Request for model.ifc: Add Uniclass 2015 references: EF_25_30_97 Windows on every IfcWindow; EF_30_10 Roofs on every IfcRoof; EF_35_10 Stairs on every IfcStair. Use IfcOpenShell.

First a look at what the model holds.

```python
import ifcopenshell

model = ifcopenshell.open("model.ifc")
print(model.schema)
print("classifications:", [c.Name for c in model.by_type("IfcClassification")])
for ifc_class in ("IfcDoor", "IfcRoof", "IfcStair", "IfcWall", "IfcWindow"):
    print(ifc_class, len(model.by_type(ifc_class)))
```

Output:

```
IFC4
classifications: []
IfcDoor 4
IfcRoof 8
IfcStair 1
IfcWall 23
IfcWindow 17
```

```python
import ifcopenshell
import ifcopenshell.api.classification

model = ifcopenshell.open("model.ifc")

system = ifcopenshell.api.classification.add_classification(model, classification="Uniclass 2015")

codes = {
    "IfcWindow": ("EF_25_30_97", "Windows"),
    "IfcRoof": ("EF_30_10", "Roofs"),
    "IfcStair": ("EF_35_10", "Stairs"),
}
for ifc_class, (code, name) in codes.items():
    products = model.by_type(ifc_class)
    ifcopenshell.api.classification.add_reference(
        model, products=products, classification=system, identification=code, name=name
    )
    print(code, len(products))

model.write("model_edited.ifc")
```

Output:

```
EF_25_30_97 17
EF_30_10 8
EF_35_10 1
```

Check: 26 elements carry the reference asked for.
